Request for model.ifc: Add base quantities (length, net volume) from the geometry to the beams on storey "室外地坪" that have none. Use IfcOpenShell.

First a look at what the model holds.

```python
import ifcopenshell
import ifcopenshell.util.element
import ifcopenshell.util.unit

model = ifcopenshell.open("model.ifc")
print(model.schema)
for unit_type in ("LENGTHUNIT", "AREAUNIT", "VOLUMEUNIT"):
    print(unit_type, ifcopenshell.util.unit.calculate_unit_scale(model, unit_type))
storey = next(s for s in model.by_type("IfcBuildingStorey") if s.Name == "室外地坪")
beams = [e for e in ifcopenshell.util.element.get_decomposition(storey) if e.is_a("IfcBeam")]
for e in sorted(beams, key=lambda e: e.id()):
    print(e.id(), e.is_a(), e.Name, list(ifcopenshell.util.element.get_psets(e, qtos_only=True)), sep=" | ")
```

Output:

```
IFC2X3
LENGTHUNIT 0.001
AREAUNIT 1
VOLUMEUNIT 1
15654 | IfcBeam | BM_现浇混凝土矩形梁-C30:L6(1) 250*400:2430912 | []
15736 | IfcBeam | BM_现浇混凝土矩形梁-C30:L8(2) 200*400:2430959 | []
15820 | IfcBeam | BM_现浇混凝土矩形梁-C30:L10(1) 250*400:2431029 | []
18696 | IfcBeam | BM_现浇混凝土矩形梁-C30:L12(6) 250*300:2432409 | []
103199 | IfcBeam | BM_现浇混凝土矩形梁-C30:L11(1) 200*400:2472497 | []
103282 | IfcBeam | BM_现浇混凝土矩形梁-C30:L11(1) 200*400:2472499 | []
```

```python
import ifcopenshell
import ifcopenshell.api.pset
import ifcopenshell.geom
import ifcopenshell.util.element
import ifcopenshell.util.shape
import ifcopenshell.util.unit

model = ifcopenshell.open("model.ifc")
unit_scale = ifcopenshell.util.unit.calculate_unit_scale(model)
volume_scale = ifcopenshell.util.unit.calculate_unit_scale(model, "VOLUMEUNIT")
settings = ifcopenshell.geom.settings()

storey = next(s for s in model.by_type("IfcBuildingStorey") if s.Name == "室外地坪")
beams = [e for e in ifcopenshell.util.element.get_decomposition(storey) if e.is_a("IfcBeam")]

for e in sorted(beams, key=lambda e: e.id()):
    if ifcopenshell.util.element.get_psets(e, qtos_only=True, should_inherit=False):
        continue
    # Geometry comes back in metres, in the element's own axes.
    shape = ifcopenshell.geom.create_shape(settings, e)
    values = {
        "Length": ifcopenshell.util.shape.get_max_xyz(shape.geometry) / unit_scale,
        "NetVolume": ifcopenshell.util.shape.get_volume(shape.geometry) / volume_scale,
    }
    qto = ifcopenshell.api.pset.add_qto(model, product=e, name="BaseQuantities")
    ifcopenshell.api.pset.edit_qto(model, qto=qto, properties=values)
    print(e.id(), {k: round(v, 3) for k, v in values.items()})

model.write("model_edited.ifc")
```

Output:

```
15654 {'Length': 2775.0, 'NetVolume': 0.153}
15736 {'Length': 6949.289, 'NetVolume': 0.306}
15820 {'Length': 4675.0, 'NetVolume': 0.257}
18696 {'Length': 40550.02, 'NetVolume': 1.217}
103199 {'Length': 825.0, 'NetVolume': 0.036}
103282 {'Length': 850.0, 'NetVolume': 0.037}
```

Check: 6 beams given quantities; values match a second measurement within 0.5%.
